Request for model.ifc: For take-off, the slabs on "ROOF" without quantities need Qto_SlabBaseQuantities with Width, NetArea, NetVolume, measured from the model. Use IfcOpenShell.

First a look at what the model holds.

```python
import ifcopenshell
import ifcopenshell.util.element
import ifcopenshell.util.unit

model = ifcopenshell.open("model.ifc")
print(model.schema)
for unit_type in ("LENGTHUNIT", "AREAUNIT", "VOLUMEUNIT"):
    print(unit_type, ifcopenshell.util.unit.calculate_unit_scale(model, unit_type))
storey = next(s for s in model.by_type("IfcBuildingStorey") if s.Name == "ROOF")
slabs = [e for e in ifcopenshell.util.element.get_decomposition(storey) if e.is_a("IfcSlab")]
for e in sorted(slabs, key=lambda e: e.id()):
    print(e.id(), e.is_a(), e.Name, list(ifcopenshell.util.element.get_psets(e, qtos_only=True)), sep=" | ")
```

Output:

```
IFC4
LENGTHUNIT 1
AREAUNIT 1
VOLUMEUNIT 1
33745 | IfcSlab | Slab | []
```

```python
import ifcopenshell
import ifcopenshell.api.pset
import ifcopenshell.geom
import ifcopenshell.util.element
import ifcopenshell.util.shape
import ifcopenshell.util.unit

model = ifcopenshell.open("model.ifc")
unit_scale = ifcopenshell.util.unit.calculate_unit_scale(model)
area_scale = ifcopenshell.util.unit.calculate_unit_scale(model, "AREAUNIT")
volume_scale = ifcopenshell.util.unit.calculate_unit_scale(model, "VOLUMEUNIT")
settings = ifcopenshell.geom.settings()

storey = next(s for s in model.by_type("IfcBuildingStorey") if s.Name == "ROOF")
slabs = [e for e in ifcopenshell.util.element.get_decomposition(storey) if e.is_a("IfcSlab")]

for e in sorted(slabs, key=lambda e: e.id()):
    if ifcopenshell.util.element.get_psets(e, qtos_only=True, should_inherit=False):
        continue
    # Geometry comes back in metres, in the element's own axes.
    shape = ifcopenshell.geom.create_shape(settings, e)
    values = {
        "Width": ifcopenshell.util.shape.get_z(shape.geometry) / unit_scale,
        "NetArea": ifcopenshell.util.shape.get_footprint_area(shape.geometry) / area_scale,
        "NetVolume": ifcopenshell.util.shape.get_volume(shape.geometry) / volume_scale,
    }
    qto = ifcopenshell.api.pset.add_qto(model, product=e, name="Qto_SlabBaseQuantities")
    ifcopenshell.api.pset.edit_qto(model, qto=qto, properties=values)
    print(e.id(), {k: round(v, 3) for k, v in values.items()})

model.write("model_v2.ifc")
```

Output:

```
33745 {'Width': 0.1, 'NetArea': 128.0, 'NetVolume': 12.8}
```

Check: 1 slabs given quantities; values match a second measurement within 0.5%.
